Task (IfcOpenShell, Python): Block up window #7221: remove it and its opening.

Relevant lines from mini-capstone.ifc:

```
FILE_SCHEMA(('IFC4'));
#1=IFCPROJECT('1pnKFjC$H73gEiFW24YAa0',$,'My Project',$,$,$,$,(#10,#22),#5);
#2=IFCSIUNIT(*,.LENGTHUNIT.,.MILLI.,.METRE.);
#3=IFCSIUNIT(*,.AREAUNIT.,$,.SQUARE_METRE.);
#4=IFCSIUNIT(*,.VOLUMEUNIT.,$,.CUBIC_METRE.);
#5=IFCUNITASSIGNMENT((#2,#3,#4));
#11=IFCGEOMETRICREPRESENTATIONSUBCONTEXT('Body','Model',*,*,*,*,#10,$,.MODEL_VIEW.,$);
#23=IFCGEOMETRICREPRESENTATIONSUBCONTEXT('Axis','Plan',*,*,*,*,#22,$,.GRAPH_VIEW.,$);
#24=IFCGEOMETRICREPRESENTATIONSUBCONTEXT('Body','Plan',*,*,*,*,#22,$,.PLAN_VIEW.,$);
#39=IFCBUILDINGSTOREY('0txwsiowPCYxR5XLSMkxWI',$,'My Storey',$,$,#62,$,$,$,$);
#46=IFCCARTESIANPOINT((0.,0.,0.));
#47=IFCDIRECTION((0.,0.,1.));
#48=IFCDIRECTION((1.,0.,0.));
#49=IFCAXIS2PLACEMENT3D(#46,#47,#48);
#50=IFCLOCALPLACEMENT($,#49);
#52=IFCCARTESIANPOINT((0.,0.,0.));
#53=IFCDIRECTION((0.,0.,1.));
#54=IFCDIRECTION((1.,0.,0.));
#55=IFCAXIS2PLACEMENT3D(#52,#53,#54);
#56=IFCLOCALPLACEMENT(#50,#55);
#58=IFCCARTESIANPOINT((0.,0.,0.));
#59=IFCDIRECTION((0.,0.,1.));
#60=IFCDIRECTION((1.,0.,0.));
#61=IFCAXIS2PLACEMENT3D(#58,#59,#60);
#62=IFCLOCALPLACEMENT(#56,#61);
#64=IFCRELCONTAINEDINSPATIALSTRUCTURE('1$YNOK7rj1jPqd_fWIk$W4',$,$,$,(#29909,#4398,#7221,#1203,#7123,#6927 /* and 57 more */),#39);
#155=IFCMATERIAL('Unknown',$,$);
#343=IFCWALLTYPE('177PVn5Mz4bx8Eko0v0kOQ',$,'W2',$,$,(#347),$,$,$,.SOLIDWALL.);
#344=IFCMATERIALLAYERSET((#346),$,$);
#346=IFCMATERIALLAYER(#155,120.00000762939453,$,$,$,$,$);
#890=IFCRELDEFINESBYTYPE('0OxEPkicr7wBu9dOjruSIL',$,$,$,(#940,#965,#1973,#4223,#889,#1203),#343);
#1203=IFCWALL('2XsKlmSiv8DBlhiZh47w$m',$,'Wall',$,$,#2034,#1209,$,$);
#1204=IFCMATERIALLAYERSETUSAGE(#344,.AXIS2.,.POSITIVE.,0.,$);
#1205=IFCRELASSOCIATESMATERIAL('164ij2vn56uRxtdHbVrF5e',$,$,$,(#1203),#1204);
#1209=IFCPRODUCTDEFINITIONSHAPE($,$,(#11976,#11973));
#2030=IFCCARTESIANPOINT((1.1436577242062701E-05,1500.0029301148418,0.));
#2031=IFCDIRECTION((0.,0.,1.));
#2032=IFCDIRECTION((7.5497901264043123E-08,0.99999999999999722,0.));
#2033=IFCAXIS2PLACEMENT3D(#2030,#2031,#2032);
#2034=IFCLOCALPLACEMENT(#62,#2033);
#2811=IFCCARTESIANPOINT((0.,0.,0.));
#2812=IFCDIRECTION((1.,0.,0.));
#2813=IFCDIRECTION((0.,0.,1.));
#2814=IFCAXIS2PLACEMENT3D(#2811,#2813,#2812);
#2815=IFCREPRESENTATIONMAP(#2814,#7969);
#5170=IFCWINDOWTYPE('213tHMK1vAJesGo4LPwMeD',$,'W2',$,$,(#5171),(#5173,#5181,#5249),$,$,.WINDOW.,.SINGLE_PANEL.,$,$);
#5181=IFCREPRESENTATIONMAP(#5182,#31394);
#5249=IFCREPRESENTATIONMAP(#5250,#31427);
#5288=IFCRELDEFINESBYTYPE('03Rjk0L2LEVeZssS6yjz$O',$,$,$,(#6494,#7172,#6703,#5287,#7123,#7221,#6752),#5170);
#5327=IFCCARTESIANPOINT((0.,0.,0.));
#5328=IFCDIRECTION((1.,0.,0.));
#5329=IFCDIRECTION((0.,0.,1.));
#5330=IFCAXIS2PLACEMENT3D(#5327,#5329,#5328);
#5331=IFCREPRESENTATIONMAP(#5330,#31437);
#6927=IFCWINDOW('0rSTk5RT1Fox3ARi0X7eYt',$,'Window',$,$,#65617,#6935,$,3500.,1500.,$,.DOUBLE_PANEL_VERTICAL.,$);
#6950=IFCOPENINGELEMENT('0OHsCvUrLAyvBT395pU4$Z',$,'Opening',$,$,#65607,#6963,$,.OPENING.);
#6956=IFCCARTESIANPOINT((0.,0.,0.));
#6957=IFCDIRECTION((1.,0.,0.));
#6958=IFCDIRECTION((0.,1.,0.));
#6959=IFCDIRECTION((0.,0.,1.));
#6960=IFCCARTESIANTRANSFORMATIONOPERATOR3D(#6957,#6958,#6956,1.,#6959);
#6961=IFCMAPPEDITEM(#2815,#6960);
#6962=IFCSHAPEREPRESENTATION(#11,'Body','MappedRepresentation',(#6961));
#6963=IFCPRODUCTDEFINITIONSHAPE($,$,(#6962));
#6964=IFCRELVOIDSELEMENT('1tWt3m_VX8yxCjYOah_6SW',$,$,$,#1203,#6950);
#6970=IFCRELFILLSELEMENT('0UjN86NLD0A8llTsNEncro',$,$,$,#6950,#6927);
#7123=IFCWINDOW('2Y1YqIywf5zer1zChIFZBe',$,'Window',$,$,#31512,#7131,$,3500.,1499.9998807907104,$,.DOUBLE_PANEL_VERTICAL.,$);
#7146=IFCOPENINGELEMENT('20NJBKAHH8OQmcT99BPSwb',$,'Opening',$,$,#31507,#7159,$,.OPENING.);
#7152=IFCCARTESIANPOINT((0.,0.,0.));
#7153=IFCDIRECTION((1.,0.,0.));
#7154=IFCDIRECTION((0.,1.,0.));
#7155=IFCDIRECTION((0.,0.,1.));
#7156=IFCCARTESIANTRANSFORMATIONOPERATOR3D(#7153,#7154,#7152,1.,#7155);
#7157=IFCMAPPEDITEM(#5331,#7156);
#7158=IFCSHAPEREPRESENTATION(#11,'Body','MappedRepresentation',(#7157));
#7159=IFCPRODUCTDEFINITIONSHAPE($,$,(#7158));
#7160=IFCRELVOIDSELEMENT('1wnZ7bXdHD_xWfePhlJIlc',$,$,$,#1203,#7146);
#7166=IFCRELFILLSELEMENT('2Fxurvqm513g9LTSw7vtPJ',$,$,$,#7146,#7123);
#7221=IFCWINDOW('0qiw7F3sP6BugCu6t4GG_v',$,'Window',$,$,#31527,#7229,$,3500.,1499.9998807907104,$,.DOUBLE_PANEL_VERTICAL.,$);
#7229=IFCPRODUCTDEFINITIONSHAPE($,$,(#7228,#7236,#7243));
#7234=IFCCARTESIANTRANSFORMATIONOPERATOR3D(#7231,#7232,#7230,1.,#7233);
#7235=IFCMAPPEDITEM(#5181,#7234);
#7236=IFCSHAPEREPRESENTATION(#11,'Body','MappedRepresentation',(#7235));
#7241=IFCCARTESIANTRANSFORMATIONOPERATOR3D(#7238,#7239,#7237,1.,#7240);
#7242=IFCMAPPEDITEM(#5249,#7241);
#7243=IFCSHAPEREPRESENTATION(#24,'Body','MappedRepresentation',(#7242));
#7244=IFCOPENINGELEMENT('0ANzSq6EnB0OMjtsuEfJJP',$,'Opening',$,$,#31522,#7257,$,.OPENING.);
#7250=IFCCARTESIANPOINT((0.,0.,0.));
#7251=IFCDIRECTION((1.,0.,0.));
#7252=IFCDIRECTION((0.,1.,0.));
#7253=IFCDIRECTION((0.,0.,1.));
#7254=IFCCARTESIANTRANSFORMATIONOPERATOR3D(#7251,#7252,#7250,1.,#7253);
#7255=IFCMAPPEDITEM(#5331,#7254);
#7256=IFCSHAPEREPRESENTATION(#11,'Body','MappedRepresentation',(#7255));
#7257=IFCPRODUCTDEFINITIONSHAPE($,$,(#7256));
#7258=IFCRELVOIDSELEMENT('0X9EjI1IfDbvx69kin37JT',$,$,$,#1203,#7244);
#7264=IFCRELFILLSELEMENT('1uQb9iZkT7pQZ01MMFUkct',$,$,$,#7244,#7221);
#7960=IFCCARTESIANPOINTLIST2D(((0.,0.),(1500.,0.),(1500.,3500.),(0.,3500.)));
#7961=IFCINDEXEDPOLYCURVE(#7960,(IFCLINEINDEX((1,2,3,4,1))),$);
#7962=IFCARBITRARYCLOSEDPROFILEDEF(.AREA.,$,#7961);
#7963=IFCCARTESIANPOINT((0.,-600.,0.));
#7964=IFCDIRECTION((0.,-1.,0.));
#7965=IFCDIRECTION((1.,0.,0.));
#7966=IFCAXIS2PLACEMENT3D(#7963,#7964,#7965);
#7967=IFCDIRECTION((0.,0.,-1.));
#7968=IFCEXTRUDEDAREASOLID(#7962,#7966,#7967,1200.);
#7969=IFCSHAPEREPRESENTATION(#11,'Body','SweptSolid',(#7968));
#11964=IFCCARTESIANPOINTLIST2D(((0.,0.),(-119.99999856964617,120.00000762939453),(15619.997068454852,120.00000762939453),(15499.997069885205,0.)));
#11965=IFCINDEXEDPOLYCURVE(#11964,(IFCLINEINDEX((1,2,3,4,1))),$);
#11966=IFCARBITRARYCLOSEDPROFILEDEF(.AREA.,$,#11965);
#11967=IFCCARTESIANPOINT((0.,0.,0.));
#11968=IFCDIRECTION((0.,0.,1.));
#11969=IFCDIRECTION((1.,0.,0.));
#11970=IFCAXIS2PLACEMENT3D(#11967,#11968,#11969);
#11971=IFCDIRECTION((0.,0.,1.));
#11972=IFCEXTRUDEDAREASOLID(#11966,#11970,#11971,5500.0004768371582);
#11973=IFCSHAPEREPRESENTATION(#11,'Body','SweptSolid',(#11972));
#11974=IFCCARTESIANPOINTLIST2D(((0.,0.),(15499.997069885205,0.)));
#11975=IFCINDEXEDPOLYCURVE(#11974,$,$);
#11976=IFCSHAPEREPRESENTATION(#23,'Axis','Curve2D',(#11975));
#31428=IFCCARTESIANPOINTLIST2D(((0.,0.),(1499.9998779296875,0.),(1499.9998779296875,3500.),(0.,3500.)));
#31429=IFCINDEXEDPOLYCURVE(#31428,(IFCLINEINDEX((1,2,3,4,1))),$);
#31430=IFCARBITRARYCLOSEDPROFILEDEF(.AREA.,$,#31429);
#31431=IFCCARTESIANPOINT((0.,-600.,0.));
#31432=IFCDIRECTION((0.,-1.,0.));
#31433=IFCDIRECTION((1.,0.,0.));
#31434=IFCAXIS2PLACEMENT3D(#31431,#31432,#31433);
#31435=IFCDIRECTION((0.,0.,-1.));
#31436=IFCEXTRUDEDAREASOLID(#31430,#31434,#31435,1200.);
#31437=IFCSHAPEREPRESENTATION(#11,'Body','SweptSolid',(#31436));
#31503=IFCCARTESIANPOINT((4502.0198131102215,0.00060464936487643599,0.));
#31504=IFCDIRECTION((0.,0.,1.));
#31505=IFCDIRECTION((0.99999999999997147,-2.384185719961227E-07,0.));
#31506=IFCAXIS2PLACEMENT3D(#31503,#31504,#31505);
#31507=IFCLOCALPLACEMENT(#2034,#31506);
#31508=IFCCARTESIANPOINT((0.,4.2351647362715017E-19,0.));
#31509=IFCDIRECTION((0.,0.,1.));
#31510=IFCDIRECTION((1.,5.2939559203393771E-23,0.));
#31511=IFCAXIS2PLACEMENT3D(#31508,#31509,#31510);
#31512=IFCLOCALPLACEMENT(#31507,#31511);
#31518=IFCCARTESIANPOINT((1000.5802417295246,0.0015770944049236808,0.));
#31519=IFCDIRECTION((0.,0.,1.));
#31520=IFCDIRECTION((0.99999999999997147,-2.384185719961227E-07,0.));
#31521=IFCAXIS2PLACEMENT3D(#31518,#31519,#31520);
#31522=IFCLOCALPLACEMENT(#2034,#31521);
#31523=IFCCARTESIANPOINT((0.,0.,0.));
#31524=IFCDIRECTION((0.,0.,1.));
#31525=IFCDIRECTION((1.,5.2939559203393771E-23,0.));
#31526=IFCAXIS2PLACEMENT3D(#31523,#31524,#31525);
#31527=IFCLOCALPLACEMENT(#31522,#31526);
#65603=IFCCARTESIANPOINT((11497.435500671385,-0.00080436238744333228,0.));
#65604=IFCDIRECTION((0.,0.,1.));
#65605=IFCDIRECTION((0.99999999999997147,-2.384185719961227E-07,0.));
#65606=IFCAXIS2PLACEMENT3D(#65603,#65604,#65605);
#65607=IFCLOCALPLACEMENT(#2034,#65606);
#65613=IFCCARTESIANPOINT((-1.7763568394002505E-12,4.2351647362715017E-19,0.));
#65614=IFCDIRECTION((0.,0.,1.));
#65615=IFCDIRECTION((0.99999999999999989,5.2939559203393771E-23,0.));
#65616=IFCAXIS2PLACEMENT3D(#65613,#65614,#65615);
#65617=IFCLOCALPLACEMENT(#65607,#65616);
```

```python
import ifcopenshell
import ifcopenshell.api.feature
import ifcopenshell.api.root
import ifcopenshell.geom
import ifcopenshell.util.shape

model = ifcopenshell.open("mini-capstone.ifc")
settings = ifcopenshell.geom.settings()


def volume(element):
    """Net volume in cubic metres, openings subtracted."""
    shape = ifcopenshell.geom.create_shape(settings, element)
    return ifcopenshell.util.shape.get_volume(shape.geometry)


window = model.by_guid("0qiw7F3sP6BugCu6t4GG_v")
opening = window.FillsVoids[0].RelatingOpeningElement
wall = opening.VoidsElements[0].RelatingBuildingElement
before = volume(wall)

ifcopenshell.api.root.remove_product(model, product=window)
ifcopenshell.api.feature.remove_feature(model, feature=opening)

after = volume(wall)

print(f"wall volume {before:.3f} -> {after:.3f} m3")

model.write("mini-capstone_rev.ifc")
```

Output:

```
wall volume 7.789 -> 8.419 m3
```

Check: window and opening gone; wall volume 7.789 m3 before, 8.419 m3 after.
